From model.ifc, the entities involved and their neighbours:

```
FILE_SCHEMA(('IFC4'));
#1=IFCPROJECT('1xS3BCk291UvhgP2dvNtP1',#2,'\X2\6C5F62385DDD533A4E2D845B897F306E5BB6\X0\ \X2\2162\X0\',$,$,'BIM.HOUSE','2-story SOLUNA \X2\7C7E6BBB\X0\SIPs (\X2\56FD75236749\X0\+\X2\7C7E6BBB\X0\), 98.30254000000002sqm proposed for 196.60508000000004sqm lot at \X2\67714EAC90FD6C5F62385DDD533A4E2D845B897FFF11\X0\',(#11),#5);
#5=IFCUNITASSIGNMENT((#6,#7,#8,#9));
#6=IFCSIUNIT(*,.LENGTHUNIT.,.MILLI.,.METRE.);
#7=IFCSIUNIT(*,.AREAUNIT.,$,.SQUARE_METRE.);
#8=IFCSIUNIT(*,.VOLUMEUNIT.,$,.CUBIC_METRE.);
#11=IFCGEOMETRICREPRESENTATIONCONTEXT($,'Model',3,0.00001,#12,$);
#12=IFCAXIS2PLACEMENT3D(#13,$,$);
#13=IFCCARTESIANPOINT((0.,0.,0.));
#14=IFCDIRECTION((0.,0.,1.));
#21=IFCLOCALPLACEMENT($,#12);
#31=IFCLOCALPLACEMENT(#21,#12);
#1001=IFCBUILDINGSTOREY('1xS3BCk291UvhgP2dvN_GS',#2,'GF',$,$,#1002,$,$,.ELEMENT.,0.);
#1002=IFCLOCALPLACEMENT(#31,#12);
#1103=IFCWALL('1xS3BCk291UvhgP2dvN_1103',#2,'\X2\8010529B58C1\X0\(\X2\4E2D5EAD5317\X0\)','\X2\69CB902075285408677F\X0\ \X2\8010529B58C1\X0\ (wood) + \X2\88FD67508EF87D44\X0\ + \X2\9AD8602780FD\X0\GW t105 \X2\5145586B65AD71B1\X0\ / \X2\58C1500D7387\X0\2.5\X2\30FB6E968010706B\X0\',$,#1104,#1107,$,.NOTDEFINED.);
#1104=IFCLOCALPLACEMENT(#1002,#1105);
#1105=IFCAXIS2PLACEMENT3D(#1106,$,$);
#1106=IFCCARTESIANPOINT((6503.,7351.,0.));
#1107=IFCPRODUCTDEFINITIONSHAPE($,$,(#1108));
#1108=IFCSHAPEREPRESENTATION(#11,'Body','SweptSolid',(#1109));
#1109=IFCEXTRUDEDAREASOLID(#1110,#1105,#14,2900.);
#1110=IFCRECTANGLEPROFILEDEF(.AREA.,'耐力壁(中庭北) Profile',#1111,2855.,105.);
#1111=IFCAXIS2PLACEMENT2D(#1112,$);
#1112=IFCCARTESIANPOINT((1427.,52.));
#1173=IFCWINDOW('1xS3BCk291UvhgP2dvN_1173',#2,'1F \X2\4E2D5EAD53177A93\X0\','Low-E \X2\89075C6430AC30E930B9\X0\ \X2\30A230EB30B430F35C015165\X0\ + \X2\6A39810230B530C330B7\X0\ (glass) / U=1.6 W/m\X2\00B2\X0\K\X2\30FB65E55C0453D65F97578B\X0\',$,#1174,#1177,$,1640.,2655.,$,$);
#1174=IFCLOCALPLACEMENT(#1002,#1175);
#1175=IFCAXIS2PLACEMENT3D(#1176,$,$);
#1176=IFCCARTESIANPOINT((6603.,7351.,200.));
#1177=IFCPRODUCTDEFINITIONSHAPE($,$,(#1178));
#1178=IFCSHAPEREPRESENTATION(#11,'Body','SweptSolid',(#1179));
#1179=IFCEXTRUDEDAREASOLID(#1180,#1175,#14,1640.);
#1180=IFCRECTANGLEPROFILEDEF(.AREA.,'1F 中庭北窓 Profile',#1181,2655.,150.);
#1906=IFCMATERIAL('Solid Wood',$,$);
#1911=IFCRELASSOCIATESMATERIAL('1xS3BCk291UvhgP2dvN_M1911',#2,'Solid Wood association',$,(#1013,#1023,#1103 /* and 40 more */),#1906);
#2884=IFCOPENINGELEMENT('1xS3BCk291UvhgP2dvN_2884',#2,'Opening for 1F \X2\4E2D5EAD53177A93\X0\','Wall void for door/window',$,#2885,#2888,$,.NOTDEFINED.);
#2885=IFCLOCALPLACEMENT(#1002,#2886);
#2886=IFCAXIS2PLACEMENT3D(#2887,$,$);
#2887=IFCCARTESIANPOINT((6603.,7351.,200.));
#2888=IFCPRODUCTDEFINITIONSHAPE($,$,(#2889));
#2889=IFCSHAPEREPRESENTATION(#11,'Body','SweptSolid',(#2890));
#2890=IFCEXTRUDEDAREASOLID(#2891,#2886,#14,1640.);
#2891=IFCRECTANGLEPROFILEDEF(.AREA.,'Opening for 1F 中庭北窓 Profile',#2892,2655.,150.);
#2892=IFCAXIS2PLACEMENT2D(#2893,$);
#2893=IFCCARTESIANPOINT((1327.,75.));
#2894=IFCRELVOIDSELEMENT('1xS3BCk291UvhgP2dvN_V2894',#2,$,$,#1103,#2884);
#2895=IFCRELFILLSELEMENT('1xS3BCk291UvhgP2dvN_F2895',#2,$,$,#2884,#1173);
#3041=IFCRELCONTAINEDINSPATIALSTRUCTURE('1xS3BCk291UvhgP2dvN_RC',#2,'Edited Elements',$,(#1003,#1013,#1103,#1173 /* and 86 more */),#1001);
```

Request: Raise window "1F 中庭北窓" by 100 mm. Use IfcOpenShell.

```python
import numpy as np
import ifcopenshell
import ifcopenshell.api.geometry
import ifcopenshell.util.placement
import ifcopenshell.util.unit

model = ifcopenshell.open("model.ifc")
unit_scale = ifcopenshell.util.unit.calculate_unit_scale(model)

window = model.by_id(1173)
opening = window.FillsVoids[0].RelatingOpeningElement
dz = 0.1 / unit_scale

shift = np.array([0.0, 0.0, dz])
# The window is not placed relative to its opening, so move both.
for product in (opening, window):
    matrix = ifcopenshell.util.placement.get_local_placement(product.ObjectPlacement)
    matrix[:3, 3] += shift
    ifcopenshell.api.geometry.edit_object_placement(model, product=product, matrix=matrix, is_si=False)

print(f"moved by {dz * unit_scale:+.3f} m")

model.write("model_rev.ifc")
```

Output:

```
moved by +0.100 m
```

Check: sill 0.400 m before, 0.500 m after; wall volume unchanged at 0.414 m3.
